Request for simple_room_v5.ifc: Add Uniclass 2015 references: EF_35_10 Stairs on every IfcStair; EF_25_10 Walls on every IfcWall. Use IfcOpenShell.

First a look at what the model holds.

```python
import ifcopenshell

model = ifcopenshell.open("simple_room_v5.ifc")
print(model.schema)
print("classifications:", [c.Name for c in model.by_type("IfcClassification")])
for ifc_class in ("IfcDoor", "IfcRoof", "IfcStair", "IfcWall", "IfcWindow"):
    print(ifc_class, len(model.by_type(ifc_class)))
```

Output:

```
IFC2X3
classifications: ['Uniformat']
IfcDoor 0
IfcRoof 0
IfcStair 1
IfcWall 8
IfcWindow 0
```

```python
import ifcopenshell
import ifcopenshell.api.classification

model = ifcopenshell.open("simple_room_v5.ifc")

# IFC2X3 requires Source and Edition and has no link from the project to the system.
system = model.create_entity("IfcClassification", Source="NBS", Edition="2015", Name="Uniclass 2015")

codes = {
    "IfcStair": ("EF_35_10", "Stairs"),
    "IfcWall": ("EF_25_10", "Walls"),
}
for ifc_class, (code, name) in codes.items():
    products = model.by_type(ifc_class)
    ifcopenshell.api.classification.add_reference(
        model, products=products, classification=system, identification=code, name=name
    )
    print(code, len(products))

model.write("simple_room_v5_updated.ifc")
```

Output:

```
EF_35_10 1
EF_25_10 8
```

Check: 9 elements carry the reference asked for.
